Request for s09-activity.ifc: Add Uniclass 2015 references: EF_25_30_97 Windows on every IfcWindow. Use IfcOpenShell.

First a look at what the model holds.

```python
import ifcopenshell

model = ifcopenshell.open("s09-activity.ifc")
print(model.schema)
print("classifications:", [c.Name for c in model.by_type("IfcClassification")])
for ifc_class in ("IfcDoor", "IfcRoof", "IfcStair", "IfcWall", "IfcWindow"):
    print(ifc_class, len(model.by_type(ifc_class)))
```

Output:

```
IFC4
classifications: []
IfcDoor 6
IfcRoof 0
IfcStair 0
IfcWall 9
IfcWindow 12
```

```python
import ifcopenshell
import ifcopenshell.api.classification

model = ifcopenshell.open("s09-activity.ifc")

system = ifcopenshell.api.classification.add_classification(model, classification="Uniclass 2015")

codes = {
    "IfcWindow": ("EF_25_30_97", "Windows"),
}
for ifc_class, (code, name) in codes.items():
    products = model.by_type(ifc_class)
    ifcopenshell.api.classification.add_reference(
        model, products=products, classification=system, identification=code, name=name
    )
    print(code, len(products))

model.write("s09-activity_updated.ifc")
```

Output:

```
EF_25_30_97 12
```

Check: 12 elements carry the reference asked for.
